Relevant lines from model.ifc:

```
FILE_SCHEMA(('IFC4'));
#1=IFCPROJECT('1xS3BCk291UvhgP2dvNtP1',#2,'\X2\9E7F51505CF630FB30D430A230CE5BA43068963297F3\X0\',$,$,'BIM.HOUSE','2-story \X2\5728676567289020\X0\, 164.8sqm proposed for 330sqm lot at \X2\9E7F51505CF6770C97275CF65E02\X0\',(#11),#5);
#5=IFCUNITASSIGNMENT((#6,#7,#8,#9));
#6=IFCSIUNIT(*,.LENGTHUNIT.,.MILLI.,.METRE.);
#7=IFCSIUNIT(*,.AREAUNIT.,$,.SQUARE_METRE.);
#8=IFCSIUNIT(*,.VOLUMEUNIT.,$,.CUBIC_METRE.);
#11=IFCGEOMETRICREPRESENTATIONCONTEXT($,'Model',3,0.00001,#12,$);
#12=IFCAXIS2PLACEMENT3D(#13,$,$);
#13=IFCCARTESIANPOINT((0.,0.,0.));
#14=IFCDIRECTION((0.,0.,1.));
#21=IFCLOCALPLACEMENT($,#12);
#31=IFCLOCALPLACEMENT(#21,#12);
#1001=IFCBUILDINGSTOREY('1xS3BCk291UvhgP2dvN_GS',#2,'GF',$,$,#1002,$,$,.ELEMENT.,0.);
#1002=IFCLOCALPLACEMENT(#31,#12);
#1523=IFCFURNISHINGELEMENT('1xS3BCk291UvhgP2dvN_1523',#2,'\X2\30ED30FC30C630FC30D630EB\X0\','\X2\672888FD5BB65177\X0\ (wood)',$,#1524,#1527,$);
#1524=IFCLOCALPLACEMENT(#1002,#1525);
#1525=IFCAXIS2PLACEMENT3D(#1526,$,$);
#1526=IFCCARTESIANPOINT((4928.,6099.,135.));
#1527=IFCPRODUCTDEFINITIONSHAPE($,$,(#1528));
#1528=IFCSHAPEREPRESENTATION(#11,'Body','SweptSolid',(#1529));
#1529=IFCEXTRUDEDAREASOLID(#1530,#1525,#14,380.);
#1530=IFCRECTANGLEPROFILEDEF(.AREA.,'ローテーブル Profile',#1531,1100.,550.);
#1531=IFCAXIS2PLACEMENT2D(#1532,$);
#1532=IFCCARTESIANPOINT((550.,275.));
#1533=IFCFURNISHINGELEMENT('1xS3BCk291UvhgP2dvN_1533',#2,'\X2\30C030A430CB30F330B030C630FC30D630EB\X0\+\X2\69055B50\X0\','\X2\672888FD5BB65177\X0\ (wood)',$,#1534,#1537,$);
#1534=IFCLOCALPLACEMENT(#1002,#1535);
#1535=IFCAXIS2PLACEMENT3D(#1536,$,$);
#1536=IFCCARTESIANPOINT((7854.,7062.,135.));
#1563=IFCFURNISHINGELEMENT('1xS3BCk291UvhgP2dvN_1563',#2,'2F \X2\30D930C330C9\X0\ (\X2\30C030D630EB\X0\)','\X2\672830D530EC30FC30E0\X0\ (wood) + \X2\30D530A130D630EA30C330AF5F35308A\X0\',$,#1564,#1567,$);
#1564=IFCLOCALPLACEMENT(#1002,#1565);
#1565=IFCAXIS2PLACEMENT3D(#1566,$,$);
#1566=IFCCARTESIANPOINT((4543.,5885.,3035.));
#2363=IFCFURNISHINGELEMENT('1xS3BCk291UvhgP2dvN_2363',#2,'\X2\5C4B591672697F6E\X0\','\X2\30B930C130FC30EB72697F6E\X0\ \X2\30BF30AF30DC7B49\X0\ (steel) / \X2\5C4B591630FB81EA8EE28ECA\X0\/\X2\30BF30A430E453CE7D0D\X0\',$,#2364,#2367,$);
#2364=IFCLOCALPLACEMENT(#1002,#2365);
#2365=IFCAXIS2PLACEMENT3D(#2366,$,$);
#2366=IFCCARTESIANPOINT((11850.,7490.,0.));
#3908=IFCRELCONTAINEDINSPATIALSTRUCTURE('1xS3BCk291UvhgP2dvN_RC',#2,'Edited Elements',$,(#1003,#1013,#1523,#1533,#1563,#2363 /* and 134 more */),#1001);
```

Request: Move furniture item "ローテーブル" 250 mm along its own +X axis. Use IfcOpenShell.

```python
import ifcopenshell
import ifcopenshell.api.geometry
import ifcopenshell.util.placement

model = ifcopenshell.open("model.ifc")

item = model.by_guid("1xS3BCk291UvhgP2dvN_1523")
matrix = ifcopenshell.util.placement.get_local_placement(item.ObjectPlacement)
matrix[:3, 3] += matrix[:3, 0] * 250.0
ifcopenshell.api.geometry.edit_object_placement(model, product=item, matrix=matrix, is_si=False)

print(ifcopenshell.util.placement.get_local_placement(item.ObjectPlacement).round(3) + 0.0)

model.write("model_edited.ifc")
```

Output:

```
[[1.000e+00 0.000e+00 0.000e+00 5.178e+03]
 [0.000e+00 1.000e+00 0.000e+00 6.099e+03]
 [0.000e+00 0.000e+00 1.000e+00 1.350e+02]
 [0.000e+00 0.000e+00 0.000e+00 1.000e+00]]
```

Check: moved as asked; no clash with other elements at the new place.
